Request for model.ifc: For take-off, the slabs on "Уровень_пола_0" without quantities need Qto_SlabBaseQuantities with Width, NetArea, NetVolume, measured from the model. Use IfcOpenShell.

First a look at what the model holds.

```python
import ifcopenshell
import ifcopenshell.util.element
import ifcopenshell.util.unit

model = ifcopenshell.open("model.ifc")
print(model.schema)
for unit_type in ("LENGTHUNIT", "AREAUNIT", "VOLUMEUNIT"):
    print(unit_type, ifcopenshell.util.unit.calculate_unit_scale(model, unit_type))
storey = next(s for s in model.by_type("IfcBuildingStorey") if s.Name == "Уровень_пола_0")
slabs = [e for e in ifcopenshell.util.element.get_decomposition(storey) if e.is_a("IfcSlab")]
for e in sorted(slabs, key=lambda e: e.id()):
    print(e.id(), e.is_a(), e.Name, list(ifcopenshell.util.element.get_psets(e, qtos_only=True)), sep=" | ")
```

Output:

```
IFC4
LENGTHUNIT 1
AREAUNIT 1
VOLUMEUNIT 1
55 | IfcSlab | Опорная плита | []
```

```python
import ifcopenshell
import ifcopenshell.api.pset
import ifcopenshell.geom
import ifcopenshell.util.element
import ifcopenshell.util.shape
import ifcopenshell.util.unit

model = ifcopenshell.open("model.ifc")
unit_scale = ifcopenshell.util.unit.calculate_unit_scale(model)
area_scale = ifcopenshell.util.unit.calculate_unit_scale(model, "AREAUNIT")
volume_scale = ifcopenshell.util.unit.calculate_unit_scale(model, "VOLUMEUNIT")
settings = ifcopenshell.geom.settings()

storey = next(s for s in model.by_type("IfcBuildingStorey") if s.Name == "Уровень_пола_0")
slabs = [e for e in ifcopenshell.util.element.get_decomposition(storey) if e.is_a("IfcSlab")]

for e in sorted(slabs, key=lambda e: e.id()):
    if ifcopenshell.util.element.get_psets(e, qtos_only=True, should_inherit=False):
        continue
    # Geometry comes back in metres, in the element's own axes.
    shape = ifcopenshell.geom.create_shape(settings, e)
    values = {
        "Width": ifcopenshell.util.shape.get_z(shape.geometry) / unit_scale,
        "NetArea": ifcopenshell.util.shape.get_footprint_area(shape.geometry) / area_scale,
        "NetVolume": ifcopenshell.util.shape.get_volume(shape.geometry) / volume_scale,
    }
    qto = ifcopenshell.api.pset.add_qto(model, product=e, name="Qto_SlabBaseQuantities")
    ifcopenshell.api.pset.edit_qto(model, qto=qto, properties=values)
    print(e.id(), {k: round(v, 3) for k, v in values.items()})

model.write("model_v2.ifc")
```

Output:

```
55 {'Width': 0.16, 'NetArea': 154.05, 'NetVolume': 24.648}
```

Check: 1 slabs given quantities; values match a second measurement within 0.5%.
